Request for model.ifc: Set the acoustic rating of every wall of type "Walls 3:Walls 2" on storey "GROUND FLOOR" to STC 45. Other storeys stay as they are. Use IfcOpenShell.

First a look at what the model holds.

```python
import ifcopenshell
import ifcopenshell.util.element

model = ifcopenshell.open("model.ifc")
print(model.schema)
storey = next(s for s in model.by_type("IfcBuildingStorey") if s.Name == "GROUND FLOOR")
walls = [e for e in ifcopenshell.util.element.get_decomposition(storey) if e.is_a("IfcWall")]
seen = {}
for e in walls:
    element_type = ifcopenshell.util.element.get_type(e)
    key = (element_type.Name if element_type != e and element_type else None, ifcopenshell.util.element.get_pset(e, "Pset_WallCommon", "AcousticRating"))
    seen[key] = seen.get(key, 0) + 1
for (name, value), count in sorted(seen.items(), key=str):
    print(count, "x", name, "|", value)
```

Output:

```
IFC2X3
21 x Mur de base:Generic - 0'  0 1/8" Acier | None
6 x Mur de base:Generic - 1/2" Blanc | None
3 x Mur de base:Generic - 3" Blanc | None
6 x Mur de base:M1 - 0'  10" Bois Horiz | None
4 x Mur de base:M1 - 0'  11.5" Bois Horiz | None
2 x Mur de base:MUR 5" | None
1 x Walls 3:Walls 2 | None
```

```python
import ifcopenshell
import ifcopenshell.api.pset
import ifcopenshell.util.element

model = ifcopenshell.open("model.ifc")

storey = next(s for s in model.by_type("IfcBuildingStorey") if s.Name == "GROUND FLOOR")
walls = [e for e in ifcopenshell.util.element.get_decomposition(storey) if e.is_a("IfcWall")]

count = 0
for e in walls:
    element_type = ifcopenshell.util.element.get_type(e)
    if element_type in (None, e) or element_type.Name != "Walls 3:Walls 2":
        continue
    # add_pset returns the element's existing set when there is one.
    pset = ifcopenshell.api.pset.add_pset(model, product=e, name="Pset_WallCommon")
    ifcopenshell.api.pset.edit_pset(model, pset=pset, properties={"AcousticRating": "STC 45"})
    count += 1

print(count, "walls updated")

model.write("model-out.ifc")
```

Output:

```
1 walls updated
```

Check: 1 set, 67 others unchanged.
